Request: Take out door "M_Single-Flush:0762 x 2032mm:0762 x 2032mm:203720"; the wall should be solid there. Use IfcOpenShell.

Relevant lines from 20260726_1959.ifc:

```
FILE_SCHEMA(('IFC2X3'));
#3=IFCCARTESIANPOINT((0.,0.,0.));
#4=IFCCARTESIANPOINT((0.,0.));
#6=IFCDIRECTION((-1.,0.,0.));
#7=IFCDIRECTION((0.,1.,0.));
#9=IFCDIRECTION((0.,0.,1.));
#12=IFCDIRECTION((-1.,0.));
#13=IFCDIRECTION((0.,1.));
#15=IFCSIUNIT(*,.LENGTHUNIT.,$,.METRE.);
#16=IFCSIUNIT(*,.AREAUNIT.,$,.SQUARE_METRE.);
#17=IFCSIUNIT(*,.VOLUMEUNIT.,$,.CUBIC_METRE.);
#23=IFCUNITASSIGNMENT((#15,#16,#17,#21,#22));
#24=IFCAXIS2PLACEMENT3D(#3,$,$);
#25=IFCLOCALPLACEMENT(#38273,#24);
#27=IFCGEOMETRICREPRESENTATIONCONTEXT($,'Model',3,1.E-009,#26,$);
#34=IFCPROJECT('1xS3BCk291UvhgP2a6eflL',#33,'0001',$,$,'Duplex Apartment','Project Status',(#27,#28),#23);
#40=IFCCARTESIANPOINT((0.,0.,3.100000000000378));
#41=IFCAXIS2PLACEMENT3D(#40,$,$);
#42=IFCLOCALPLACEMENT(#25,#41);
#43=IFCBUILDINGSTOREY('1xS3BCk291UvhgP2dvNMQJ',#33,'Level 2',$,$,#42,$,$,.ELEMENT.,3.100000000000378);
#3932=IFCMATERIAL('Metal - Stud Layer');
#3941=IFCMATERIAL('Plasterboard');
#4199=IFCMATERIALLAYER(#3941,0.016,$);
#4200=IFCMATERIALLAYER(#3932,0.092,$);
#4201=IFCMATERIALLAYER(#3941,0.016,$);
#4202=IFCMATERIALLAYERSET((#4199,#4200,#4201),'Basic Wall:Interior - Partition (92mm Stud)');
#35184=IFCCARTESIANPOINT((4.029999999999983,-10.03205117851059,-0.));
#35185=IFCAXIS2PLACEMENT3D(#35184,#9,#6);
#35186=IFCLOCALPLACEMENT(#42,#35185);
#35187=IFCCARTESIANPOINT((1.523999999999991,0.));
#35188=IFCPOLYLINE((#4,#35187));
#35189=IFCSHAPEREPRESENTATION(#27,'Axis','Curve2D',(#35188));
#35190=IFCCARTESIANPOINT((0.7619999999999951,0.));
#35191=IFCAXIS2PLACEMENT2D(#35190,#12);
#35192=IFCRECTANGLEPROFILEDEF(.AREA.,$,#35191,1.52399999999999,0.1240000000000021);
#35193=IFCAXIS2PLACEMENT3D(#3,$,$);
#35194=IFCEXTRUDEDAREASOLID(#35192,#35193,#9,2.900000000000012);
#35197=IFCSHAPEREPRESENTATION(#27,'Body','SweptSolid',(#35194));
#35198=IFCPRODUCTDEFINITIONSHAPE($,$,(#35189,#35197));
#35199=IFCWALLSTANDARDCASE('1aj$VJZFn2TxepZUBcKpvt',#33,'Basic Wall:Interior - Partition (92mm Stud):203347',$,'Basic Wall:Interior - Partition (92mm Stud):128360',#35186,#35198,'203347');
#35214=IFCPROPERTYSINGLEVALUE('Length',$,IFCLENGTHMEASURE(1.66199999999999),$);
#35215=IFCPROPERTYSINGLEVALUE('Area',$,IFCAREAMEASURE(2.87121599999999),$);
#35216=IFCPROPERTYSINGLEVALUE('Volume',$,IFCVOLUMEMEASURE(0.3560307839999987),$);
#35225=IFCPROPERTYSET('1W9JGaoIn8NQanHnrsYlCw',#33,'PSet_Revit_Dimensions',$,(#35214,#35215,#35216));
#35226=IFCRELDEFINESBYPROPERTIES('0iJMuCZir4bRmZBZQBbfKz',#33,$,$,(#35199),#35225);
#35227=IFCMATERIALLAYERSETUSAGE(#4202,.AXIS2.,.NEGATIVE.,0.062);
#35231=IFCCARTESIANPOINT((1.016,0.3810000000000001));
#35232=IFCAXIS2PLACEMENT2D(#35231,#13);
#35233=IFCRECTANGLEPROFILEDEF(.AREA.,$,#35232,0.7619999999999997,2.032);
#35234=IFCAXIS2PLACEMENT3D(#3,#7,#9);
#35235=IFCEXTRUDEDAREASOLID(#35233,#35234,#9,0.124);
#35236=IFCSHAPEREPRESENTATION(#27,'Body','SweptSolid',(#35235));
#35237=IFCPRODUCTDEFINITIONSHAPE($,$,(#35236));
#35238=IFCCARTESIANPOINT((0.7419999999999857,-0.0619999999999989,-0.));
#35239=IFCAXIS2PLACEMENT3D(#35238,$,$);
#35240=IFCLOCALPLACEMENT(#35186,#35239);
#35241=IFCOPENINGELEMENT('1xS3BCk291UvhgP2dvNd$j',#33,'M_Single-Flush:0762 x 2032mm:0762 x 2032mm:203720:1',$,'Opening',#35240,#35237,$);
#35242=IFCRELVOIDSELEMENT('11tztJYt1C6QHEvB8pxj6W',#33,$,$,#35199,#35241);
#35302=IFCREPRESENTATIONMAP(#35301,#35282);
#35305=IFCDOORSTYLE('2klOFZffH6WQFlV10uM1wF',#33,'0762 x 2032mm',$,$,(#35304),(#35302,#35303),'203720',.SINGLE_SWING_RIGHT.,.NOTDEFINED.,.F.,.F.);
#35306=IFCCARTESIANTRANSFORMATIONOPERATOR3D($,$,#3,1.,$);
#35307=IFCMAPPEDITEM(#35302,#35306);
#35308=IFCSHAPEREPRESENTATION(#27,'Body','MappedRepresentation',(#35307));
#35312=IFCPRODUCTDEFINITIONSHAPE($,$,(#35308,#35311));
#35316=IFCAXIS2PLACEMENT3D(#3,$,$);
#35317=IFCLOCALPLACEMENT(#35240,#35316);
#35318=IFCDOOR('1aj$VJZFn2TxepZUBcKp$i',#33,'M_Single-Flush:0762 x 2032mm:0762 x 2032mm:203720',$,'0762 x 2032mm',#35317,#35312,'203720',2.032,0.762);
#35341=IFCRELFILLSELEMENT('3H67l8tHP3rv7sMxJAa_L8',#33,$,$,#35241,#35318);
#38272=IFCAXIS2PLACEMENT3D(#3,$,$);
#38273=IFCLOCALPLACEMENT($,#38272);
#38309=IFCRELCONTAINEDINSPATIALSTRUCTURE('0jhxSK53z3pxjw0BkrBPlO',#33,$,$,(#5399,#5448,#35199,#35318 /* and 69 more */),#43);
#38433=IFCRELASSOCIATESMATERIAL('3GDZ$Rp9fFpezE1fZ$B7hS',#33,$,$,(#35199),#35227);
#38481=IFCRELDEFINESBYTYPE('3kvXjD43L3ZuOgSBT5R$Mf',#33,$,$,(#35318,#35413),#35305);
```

```python
import ifcopenshell
import ifcopenshell.api.feature
import ifcopenshell.api.pset
import ifcopenshell.api.root
import ifcopenshell.geom
import ifcopenshell.util.element
import ifcopenshell.util.shape
import ifcopenshell.util.unit

model = ifcopenshell.open("20260726_1959.ifc")
area_scale = ifcopenshell.util.unit.calculate_unit_scale(model, "AREAUNIT")
volume_scale = ifcopenshell.util.unit.calculate_unit_scale(model, "VOLUMEUNIT")
settings = ifcopenshell.geom.settings()


def volume(element):
    """Net volume in cubic metres, openings subtracted."""
    shape = ifcopenshell.geom.create_shape(settings, element)
    return ifcopenshell.util.shape.get_volume(shape.geometry)


door = model.by_id(35318)
opening = door.FillsVoids[0].RelatingOpeningElement
wall = opening.VoidsElements[0].RelatingBuildingElement
before = volume(wall)

ifcopenshell.api.root.remove_product(model, product=door)
ifcopenshell.api.feature.remove_feature(model, feature=opening)

after = volume(wall)
thickness = 0.124  # wall thickness in metres

# Update the wall's stored quantities.
pset = model.by_id(ifcopenshell.util.element.get_pset(wall, "PSet_Revit_Dimensions", should_inherit=False)["id"])
ifcopenshell.api.pset.edit_pset(model, pset=pset, properties={
    "Area": model.create_entity("IfcAreaMeasure", after / thickness / area_scale),
    "Volume": model.create_entity("IfcVolumeMeasure", after / volume_scale),
})

print(f"wall volume {before:.3f} -> {after:.3f} m3")

model.write("20260726_1959-out.ifc")
```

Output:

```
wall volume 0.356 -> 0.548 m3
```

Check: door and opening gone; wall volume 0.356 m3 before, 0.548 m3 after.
